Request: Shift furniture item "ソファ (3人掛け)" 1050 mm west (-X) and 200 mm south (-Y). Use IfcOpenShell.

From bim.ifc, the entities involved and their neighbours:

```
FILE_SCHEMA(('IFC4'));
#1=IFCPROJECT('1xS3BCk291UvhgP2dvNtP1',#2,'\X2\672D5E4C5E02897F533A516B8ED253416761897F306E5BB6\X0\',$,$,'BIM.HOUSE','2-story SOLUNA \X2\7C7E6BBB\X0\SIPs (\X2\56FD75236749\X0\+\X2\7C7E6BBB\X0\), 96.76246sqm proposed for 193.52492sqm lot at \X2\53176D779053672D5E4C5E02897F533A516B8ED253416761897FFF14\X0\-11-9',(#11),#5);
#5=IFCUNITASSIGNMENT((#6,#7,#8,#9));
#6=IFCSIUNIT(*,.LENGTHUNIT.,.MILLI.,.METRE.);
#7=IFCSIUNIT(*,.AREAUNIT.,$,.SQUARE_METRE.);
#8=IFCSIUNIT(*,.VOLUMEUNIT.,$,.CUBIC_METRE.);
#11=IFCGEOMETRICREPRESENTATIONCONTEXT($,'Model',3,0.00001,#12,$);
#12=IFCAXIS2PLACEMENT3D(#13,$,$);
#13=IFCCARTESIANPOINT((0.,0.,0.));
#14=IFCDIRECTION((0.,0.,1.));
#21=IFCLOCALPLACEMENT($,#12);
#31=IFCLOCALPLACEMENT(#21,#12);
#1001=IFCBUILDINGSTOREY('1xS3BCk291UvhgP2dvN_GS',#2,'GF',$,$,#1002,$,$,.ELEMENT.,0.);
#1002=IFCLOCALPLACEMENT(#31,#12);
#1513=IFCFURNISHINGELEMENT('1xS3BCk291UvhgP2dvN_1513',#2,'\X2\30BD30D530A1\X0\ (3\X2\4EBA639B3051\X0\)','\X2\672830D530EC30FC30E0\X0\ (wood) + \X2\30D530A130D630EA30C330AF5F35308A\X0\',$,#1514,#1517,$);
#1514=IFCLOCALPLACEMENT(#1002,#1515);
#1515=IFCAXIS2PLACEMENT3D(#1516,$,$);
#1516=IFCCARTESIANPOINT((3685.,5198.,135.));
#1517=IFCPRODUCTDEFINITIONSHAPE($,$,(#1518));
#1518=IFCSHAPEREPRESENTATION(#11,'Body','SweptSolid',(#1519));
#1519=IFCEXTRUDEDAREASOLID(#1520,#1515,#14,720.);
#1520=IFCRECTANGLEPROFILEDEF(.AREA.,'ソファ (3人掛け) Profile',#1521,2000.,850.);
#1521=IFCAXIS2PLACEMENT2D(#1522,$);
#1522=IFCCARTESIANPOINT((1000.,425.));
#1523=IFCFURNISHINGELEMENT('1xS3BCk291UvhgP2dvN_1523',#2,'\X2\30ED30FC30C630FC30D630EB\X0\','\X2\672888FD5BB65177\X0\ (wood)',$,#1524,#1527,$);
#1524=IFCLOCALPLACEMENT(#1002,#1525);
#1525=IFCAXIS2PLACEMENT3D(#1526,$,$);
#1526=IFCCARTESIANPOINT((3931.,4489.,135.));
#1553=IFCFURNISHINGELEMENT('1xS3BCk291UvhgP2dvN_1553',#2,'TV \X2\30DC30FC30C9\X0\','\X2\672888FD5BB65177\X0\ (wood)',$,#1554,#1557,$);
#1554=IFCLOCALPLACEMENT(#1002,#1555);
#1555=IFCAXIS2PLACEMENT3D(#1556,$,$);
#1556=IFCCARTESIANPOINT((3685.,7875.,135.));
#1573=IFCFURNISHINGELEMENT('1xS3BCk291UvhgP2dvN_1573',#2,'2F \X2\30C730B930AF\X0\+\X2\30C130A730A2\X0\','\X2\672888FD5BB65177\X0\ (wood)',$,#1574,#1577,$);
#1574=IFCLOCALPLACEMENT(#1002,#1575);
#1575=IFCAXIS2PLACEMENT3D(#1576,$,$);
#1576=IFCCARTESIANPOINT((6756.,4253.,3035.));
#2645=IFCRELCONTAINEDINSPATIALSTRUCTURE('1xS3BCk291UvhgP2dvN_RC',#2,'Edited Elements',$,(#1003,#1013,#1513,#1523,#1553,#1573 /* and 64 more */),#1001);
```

```python
import ifcopenshell
import ifcopenshell.api.geometry
import ifcopenshell.util.placement
import ifcopenshell.util.unit

model = ifcopenshell.open("bim.ifc")
unit_scale = ifcopenshell.util.unit.calculate_unit_scale(model)

item = model.by_guid("1xS3BCk291UvhgP2dvN_1513")
matrix = ifcopenshell.util.placement.get_local_placement(item.ObjectPlacement)
matrix[0, 3] -= 1.05 / unit_scale
matrix[1, 3] -= 0.2 / unit_scale
ifcopenshell.api.geometry.edit_object_placement(model, product=item, matrix=matrix, is_si=False)

print(ifcopenshell.util.placement.get_local_placement(item.ObjectPlacement).round(3) + 0.0)

model.write("bim_edited.ifc")
```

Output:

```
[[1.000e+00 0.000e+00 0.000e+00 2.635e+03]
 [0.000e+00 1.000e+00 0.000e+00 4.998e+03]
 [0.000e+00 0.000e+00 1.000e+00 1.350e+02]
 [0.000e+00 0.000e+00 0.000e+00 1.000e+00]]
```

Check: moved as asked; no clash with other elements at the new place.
